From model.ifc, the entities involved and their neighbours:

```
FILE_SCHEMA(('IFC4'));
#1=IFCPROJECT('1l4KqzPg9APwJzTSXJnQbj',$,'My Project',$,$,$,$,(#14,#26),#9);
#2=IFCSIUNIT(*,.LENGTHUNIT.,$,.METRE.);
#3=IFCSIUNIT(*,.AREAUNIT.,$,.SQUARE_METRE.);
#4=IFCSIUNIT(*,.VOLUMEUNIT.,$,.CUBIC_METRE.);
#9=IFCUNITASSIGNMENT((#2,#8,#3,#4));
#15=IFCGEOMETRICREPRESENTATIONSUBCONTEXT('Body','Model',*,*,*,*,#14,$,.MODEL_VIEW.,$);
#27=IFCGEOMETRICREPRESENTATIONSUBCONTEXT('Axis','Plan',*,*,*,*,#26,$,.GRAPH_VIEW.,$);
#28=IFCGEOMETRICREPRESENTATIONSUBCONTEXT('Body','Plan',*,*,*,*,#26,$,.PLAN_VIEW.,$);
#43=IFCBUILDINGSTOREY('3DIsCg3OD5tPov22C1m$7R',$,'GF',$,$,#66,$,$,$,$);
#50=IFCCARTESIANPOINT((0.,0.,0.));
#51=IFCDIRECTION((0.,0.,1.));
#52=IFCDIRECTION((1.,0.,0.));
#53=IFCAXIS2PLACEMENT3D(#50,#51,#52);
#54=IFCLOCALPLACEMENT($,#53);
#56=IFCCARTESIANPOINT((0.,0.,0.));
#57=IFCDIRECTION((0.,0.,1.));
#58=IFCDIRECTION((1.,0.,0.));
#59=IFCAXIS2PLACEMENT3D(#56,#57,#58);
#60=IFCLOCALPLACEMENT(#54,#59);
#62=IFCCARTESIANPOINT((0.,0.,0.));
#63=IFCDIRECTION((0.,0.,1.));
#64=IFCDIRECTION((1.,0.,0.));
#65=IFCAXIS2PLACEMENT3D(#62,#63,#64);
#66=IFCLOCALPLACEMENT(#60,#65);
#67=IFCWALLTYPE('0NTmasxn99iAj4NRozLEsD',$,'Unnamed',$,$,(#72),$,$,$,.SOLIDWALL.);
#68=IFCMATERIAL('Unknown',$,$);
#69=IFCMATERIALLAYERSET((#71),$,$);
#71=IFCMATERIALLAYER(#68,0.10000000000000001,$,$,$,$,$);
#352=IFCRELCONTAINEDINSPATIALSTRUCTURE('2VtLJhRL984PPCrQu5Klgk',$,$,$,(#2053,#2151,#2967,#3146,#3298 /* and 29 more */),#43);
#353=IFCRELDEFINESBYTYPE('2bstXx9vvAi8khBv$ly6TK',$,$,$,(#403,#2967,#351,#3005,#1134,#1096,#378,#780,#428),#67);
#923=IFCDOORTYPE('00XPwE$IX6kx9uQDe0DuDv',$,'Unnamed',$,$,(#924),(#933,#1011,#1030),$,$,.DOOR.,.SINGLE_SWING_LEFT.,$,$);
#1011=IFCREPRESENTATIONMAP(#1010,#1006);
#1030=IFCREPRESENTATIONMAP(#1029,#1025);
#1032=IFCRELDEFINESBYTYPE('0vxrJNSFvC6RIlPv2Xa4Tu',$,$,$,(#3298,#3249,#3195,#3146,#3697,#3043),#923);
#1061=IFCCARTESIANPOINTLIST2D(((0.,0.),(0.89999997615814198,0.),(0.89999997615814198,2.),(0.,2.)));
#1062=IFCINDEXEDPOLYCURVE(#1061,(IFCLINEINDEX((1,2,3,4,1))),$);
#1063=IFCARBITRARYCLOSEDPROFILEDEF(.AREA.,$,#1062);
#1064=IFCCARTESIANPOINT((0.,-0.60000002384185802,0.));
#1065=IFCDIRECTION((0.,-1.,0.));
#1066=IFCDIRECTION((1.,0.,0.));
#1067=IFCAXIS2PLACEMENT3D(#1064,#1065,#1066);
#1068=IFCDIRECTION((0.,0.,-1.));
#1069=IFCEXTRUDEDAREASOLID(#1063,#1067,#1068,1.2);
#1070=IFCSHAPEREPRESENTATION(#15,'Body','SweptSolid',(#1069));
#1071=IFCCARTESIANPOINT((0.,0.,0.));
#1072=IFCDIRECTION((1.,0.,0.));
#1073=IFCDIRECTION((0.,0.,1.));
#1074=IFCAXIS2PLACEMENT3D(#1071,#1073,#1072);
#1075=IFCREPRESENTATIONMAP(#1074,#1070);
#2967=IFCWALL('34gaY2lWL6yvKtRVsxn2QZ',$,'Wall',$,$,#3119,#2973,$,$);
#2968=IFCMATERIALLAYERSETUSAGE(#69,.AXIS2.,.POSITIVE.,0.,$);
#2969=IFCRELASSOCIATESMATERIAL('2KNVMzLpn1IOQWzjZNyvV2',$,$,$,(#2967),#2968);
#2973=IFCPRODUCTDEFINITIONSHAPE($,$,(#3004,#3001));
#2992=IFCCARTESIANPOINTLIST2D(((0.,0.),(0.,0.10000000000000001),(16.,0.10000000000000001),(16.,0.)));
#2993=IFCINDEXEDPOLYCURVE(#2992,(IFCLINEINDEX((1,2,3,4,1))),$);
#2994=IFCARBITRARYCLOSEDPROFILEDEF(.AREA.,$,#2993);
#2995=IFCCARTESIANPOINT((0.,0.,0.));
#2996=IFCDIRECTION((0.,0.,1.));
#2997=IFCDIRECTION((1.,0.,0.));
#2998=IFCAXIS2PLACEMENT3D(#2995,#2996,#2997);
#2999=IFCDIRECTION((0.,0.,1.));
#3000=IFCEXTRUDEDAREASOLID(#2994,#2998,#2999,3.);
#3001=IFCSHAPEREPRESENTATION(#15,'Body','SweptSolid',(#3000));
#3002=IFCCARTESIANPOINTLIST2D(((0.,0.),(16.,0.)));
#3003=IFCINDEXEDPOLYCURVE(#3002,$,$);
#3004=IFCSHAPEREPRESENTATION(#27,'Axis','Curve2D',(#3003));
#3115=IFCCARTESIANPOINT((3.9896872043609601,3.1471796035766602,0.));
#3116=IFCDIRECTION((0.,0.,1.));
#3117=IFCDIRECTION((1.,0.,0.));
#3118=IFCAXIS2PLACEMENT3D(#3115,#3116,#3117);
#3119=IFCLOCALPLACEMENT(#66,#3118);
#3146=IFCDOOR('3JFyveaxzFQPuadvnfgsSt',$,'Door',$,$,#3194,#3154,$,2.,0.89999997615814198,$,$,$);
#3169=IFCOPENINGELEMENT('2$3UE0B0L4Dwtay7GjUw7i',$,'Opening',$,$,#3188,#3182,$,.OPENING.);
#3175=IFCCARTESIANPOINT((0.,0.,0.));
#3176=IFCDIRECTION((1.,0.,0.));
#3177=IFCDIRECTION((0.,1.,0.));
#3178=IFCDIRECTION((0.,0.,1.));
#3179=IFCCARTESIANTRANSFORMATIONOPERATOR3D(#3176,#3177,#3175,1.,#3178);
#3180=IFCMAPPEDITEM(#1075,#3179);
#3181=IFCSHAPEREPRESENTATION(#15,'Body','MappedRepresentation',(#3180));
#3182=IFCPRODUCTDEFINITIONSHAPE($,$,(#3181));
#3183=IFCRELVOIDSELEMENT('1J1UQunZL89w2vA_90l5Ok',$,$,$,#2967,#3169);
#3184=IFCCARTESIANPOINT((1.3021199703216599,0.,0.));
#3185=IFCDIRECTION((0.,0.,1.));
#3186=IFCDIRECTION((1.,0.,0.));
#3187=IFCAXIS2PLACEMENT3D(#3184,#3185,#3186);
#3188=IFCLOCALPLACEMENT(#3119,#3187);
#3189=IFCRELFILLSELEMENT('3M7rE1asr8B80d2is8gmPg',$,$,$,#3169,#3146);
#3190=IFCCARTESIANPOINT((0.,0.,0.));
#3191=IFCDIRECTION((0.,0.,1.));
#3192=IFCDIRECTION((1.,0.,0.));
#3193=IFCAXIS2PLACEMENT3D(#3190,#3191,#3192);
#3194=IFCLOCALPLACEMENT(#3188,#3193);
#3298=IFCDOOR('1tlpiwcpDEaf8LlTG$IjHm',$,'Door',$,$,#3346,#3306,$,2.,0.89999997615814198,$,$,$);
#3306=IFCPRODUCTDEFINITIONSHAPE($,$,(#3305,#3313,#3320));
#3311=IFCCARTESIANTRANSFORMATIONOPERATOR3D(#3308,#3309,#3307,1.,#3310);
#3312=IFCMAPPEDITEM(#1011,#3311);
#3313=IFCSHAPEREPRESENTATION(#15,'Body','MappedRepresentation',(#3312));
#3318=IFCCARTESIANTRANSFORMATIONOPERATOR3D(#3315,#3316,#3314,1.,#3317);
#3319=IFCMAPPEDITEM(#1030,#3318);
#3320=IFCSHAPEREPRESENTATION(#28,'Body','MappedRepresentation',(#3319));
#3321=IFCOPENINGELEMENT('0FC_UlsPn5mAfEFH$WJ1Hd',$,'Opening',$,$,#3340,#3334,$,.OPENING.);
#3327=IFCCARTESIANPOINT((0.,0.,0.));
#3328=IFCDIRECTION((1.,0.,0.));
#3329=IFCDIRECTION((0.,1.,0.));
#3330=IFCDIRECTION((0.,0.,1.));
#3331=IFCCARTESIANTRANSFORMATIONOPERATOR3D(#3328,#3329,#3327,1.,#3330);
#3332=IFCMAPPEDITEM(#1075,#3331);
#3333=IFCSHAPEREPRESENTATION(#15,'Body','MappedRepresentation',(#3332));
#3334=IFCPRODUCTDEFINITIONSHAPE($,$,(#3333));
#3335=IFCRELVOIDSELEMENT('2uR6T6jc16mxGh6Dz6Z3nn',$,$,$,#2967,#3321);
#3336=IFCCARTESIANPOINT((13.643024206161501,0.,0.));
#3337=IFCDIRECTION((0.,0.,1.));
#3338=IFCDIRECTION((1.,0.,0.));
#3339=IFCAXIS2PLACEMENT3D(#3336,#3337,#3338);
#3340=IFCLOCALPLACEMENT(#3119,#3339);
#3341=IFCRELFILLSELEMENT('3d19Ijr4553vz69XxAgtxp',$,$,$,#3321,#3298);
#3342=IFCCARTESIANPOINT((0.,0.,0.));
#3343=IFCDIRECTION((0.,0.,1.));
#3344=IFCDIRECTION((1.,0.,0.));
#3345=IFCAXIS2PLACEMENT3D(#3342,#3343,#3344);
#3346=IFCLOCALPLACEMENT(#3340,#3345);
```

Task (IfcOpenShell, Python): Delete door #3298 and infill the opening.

```python
import ifcopenshell
import ifcopenshell.api.feature
import ifcopenshell.api.root
import ifcopenshell.geom
import ifcopenshell.util.shape

model = ifcopenshell.open("model.ifc")
settings = ifcopenshell.geom.settings()


def volume(element):
    """Net volume in cubic metres, openings subtracted."""
    shape = ifcopenshell.geom.create_shape(settings, element)
    return ifcopenshell.util.shape.get_volume(shape.geometry)


door = model.by_guid("1tlpiwcpDEaf8LlTG$IjHm")
opening = door.FillsVoids[0].RelatingOpeningElement
wall = opening.VoidsElements[0].RelatingBuildingElement
before = volume(wall)

ifcopenshell.api.root.remove_product(model, product=door)
ifcopenshell.api.feature.remove_feature(model, feature=opening)

after = volume(wall)

print(f"wall volume {before:.3f} -> {after:.3f} m3")

model.write("model_rev.ifc")
```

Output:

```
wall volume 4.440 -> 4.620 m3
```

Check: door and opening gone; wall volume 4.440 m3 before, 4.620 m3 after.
